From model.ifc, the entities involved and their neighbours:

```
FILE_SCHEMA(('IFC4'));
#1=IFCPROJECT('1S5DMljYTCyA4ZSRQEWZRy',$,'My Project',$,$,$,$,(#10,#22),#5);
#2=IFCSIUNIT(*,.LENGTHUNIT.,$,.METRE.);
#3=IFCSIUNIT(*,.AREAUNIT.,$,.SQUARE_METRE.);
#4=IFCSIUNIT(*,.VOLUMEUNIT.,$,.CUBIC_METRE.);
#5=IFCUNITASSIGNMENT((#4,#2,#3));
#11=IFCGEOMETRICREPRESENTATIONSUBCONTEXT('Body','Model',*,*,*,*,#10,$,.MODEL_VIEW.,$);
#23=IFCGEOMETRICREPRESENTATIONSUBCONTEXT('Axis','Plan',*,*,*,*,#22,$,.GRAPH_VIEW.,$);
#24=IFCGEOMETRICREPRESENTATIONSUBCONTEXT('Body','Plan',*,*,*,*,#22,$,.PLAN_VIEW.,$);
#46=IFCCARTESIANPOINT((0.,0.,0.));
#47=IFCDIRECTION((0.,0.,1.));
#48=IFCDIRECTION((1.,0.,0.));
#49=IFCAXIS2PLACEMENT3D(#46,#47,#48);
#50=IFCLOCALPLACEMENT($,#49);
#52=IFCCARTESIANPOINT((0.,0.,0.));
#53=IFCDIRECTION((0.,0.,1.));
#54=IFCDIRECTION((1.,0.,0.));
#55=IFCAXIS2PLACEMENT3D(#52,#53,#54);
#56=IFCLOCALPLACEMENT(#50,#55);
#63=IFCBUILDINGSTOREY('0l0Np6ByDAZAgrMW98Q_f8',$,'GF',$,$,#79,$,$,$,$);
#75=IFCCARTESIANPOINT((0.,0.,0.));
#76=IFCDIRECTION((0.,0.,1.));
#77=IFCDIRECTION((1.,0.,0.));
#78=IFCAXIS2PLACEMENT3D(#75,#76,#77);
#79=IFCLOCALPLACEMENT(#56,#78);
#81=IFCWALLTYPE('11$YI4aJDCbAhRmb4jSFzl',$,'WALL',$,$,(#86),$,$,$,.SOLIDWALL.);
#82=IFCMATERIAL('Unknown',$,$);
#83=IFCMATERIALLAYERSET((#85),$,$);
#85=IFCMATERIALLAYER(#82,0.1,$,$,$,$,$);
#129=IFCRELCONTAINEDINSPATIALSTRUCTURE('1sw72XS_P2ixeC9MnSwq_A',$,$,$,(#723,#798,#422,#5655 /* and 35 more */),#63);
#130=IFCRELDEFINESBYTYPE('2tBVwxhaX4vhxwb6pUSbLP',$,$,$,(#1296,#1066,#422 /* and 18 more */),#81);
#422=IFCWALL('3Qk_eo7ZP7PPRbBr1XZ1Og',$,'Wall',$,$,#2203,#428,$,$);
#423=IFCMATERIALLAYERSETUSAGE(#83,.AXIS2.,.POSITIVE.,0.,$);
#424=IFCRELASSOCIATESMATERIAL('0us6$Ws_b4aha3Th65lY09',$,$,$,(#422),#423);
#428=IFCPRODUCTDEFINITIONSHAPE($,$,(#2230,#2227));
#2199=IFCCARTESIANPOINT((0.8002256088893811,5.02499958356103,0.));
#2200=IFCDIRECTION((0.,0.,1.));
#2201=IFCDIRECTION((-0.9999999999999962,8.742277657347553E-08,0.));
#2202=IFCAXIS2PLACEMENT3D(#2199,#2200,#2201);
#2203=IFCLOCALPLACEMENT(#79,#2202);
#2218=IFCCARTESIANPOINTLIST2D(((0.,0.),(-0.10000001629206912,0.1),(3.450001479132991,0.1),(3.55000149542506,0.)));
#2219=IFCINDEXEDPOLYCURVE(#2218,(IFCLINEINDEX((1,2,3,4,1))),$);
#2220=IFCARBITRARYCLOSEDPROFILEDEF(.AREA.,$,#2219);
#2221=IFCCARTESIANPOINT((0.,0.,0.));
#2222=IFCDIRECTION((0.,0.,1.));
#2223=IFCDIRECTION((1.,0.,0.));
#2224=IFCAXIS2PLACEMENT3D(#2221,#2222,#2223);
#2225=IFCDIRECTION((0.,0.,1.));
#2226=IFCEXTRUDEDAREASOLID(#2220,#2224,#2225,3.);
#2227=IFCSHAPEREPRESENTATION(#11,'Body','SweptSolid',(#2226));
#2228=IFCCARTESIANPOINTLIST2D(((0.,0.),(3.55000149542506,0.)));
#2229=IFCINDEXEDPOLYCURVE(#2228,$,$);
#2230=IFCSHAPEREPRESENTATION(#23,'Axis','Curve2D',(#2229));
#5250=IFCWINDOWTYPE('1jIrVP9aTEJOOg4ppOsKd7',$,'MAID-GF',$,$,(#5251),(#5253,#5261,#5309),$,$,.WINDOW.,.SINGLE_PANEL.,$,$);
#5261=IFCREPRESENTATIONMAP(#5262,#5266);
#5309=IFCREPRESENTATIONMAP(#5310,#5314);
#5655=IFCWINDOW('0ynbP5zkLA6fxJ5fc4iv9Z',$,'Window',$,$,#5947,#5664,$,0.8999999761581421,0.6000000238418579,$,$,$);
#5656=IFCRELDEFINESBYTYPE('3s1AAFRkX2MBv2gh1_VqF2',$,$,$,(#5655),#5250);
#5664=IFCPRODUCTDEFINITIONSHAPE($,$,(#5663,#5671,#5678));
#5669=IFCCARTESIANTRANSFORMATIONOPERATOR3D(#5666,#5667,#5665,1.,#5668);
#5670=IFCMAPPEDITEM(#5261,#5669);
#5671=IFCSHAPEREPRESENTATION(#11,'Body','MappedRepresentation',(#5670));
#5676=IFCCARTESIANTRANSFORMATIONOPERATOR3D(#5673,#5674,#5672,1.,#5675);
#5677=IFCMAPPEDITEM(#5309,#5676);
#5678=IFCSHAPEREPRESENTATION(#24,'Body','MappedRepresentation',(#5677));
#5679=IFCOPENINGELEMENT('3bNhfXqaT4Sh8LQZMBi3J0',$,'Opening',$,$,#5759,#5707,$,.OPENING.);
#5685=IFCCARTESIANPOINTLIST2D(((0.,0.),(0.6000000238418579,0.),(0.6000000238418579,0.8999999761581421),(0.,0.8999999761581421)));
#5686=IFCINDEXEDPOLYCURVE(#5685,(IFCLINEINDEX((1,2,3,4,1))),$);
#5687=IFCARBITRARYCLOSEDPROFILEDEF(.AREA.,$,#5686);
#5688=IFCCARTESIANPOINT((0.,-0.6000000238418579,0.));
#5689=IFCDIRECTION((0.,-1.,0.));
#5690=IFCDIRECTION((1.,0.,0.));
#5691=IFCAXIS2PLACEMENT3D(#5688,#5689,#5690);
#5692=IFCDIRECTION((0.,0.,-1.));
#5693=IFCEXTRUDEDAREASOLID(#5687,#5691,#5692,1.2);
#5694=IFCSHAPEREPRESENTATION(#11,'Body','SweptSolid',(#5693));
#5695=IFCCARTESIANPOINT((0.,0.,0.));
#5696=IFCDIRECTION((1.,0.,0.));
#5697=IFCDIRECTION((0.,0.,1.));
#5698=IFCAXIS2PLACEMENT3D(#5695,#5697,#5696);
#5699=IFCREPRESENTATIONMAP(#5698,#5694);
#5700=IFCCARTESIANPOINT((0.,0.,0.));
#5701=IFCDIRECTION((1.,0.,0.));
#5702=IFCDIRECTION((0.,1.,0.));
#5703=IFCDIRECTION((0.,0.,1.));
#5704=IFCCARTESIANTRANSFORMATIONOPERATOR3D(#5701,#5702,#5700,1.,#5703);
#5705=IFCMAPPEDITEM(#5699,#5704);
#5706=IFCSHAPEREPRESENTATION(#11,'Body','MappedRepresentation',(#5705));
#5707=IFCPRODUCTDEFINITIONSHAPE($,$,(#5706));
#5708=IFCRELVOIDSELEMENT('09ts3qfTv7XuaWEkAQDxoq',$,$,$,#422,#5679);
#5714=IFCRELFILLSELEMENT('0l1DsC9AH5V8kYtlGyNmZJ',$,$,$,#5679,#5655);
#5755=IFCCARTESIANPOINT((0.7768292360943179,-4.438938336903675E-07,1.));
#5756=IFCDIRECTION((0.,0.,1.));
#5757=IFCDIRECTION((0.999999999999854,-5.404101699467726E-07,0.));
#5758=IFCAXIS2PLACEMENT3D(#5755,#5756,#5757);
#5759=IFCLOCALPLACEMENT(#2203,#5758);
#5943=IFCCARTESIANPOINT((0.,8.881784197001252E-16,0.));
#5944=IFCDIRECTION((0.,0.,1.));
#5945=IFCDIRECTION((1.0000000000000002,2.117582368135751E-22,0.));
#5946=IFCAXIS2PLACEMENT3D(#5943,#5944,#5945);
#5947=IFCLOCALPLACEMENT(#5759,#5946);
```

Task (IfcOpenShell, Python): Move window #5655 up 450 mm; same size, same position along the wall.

```python
import numpy as np
import ifcopenshell
import ifcopenshell.api.geometry
import ifcopenshell.util.placement
import ifcopenshell.util.unit

model = ifcopenshell.open("model.ifc")
unit_scale = ifcopenshell.util.unit.calculate_unit_scale(model)

window = model.by_id(5655)
opening = window.FillsVoids[0].RelatingOpeningElement
dz = 0.45 / unit_scale

shift = np.array([0.0, 0.0, dz])
# The window is placed relative to its opening, so it follows when the opening moves.
matrix = ifcopenshell.util.placement.get_local_placement(opening.ObjectPlacement)
matrix[:3, 3] += shift
ifcopenshell.api.geometry.edit_object_placement(
    model, product=opening, matrix=matrix, is_si=False, should_transform_children=True
)

print(f"moved by {dz * unit_scale:+.3f} m")

model.write("model_edited.ifc")
```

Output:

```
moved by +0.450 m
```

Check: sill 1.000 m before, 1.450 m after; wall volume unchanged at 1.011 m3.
